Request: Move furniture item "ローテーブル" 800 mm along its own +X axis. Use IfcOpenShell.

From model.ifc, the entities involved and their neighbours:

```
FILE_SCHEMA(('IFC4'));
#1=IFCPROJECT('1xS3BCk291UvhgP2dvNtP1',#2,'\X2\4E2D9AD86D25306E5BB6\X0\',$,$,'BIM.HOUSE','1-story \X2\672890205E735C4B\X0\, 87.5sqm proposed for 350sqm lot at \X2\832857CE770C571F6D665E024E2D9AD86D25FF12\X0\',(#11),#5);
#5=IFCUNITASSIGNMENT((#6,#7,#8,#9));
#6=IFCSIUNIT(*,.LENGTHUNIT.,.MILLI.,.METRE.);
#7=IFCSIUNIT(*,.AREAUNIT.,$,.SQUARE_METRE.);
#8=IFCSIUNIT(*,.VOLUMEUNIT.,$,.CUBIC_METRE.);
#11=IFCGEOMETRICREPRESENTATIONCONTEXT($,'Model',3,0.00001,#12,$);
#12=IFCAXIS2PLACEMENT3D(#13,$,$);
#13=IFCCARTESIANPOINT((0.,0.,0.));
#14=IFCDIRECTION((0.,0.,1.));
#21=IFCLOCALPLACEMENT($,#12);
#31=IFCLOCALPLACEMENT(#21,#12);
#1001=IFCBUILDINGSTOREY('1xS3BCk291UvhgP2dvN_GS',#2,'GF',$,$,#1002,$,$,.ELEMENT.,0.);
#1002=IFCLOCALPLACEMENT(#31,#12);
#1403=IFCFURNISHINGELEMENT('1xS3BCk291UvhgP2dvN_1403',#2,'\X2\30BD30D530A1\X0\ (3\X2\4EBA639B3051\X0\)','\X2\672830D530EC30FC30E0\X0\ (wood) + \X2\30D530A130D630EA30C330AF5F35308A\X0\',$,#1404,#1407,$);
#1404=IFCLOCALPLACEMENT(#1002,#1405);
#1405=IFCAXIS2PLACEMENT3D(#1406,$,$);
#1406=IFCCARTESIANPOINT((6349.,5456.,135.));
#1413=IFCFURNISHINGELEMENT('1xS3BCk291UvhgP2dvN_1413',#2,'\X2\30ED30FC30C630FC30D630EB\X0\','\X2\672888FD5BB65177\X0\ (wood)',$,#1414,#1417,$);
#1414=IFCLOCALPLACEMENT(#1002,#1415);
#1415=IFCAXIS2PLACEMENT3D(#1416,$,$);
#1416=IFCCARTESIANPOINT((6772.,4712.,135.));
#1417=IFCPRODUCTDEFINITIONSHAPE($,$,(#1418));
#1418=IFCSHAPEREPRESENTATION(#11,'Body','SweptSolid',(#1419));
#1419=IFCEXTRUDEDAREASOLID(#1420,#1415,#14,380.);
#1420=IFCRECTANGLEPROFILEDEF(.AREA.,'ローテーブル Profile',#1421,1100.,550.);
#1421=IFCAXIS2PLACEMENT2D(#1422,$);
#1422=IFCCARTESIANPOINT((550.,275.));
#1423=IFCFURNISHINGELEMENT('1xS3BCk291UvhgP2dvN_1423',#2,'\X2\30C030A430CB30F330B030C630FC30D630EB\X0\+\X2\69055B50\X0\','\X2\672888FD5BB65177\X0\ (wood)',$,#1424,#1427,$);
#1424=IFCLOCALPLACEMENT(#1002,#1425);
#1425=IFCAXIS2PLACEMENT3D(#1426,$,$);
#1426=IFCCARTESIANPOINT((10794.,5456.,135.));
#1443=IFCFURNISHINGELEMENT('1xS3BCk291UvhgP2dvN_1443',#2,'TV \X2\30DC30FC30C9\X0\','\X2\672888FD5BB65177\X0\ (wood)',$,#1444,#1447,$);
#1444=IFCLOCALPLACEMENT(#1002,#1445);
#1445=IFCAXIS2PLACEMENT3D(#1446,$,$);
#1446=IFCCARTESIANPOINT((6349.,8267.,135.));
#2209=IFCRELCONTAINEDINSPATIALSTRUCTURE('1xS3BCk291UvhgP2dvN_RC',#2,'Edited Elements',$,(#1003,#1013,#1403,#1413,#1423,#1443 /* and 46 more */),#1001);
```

```python
import ifcopenshell
import ifcopenshell.api.geometry
import ifcopenshell.util.placement

model = ifcopenshell.open("model.ifc")

item = model.by_guid("1xS3BCk291UvhgP2dvN_1413")
matrix = ifcopenshell.util.placement.get_local_placement(item.ObjectPlacement)
matrix[:3, 3] += matrix[:3, 0] * 800.0
ifcopenshell.api.geometry.edit_object_placement(model, product=item, matrix=matrix, is_si=False)

print(ifcopenshell.util.placement.get_local_placement(item.ObjectPlacement).round(3) + 0.0)

model.write("model_v2.ifc")
```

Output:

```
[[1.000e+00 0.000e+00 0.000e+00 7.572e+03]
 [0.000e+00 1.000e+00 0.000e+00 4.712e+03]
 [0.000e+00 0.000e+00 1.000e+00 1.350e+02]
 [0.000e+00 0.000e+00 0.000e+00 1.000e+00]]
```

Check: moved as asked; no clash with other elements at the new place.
